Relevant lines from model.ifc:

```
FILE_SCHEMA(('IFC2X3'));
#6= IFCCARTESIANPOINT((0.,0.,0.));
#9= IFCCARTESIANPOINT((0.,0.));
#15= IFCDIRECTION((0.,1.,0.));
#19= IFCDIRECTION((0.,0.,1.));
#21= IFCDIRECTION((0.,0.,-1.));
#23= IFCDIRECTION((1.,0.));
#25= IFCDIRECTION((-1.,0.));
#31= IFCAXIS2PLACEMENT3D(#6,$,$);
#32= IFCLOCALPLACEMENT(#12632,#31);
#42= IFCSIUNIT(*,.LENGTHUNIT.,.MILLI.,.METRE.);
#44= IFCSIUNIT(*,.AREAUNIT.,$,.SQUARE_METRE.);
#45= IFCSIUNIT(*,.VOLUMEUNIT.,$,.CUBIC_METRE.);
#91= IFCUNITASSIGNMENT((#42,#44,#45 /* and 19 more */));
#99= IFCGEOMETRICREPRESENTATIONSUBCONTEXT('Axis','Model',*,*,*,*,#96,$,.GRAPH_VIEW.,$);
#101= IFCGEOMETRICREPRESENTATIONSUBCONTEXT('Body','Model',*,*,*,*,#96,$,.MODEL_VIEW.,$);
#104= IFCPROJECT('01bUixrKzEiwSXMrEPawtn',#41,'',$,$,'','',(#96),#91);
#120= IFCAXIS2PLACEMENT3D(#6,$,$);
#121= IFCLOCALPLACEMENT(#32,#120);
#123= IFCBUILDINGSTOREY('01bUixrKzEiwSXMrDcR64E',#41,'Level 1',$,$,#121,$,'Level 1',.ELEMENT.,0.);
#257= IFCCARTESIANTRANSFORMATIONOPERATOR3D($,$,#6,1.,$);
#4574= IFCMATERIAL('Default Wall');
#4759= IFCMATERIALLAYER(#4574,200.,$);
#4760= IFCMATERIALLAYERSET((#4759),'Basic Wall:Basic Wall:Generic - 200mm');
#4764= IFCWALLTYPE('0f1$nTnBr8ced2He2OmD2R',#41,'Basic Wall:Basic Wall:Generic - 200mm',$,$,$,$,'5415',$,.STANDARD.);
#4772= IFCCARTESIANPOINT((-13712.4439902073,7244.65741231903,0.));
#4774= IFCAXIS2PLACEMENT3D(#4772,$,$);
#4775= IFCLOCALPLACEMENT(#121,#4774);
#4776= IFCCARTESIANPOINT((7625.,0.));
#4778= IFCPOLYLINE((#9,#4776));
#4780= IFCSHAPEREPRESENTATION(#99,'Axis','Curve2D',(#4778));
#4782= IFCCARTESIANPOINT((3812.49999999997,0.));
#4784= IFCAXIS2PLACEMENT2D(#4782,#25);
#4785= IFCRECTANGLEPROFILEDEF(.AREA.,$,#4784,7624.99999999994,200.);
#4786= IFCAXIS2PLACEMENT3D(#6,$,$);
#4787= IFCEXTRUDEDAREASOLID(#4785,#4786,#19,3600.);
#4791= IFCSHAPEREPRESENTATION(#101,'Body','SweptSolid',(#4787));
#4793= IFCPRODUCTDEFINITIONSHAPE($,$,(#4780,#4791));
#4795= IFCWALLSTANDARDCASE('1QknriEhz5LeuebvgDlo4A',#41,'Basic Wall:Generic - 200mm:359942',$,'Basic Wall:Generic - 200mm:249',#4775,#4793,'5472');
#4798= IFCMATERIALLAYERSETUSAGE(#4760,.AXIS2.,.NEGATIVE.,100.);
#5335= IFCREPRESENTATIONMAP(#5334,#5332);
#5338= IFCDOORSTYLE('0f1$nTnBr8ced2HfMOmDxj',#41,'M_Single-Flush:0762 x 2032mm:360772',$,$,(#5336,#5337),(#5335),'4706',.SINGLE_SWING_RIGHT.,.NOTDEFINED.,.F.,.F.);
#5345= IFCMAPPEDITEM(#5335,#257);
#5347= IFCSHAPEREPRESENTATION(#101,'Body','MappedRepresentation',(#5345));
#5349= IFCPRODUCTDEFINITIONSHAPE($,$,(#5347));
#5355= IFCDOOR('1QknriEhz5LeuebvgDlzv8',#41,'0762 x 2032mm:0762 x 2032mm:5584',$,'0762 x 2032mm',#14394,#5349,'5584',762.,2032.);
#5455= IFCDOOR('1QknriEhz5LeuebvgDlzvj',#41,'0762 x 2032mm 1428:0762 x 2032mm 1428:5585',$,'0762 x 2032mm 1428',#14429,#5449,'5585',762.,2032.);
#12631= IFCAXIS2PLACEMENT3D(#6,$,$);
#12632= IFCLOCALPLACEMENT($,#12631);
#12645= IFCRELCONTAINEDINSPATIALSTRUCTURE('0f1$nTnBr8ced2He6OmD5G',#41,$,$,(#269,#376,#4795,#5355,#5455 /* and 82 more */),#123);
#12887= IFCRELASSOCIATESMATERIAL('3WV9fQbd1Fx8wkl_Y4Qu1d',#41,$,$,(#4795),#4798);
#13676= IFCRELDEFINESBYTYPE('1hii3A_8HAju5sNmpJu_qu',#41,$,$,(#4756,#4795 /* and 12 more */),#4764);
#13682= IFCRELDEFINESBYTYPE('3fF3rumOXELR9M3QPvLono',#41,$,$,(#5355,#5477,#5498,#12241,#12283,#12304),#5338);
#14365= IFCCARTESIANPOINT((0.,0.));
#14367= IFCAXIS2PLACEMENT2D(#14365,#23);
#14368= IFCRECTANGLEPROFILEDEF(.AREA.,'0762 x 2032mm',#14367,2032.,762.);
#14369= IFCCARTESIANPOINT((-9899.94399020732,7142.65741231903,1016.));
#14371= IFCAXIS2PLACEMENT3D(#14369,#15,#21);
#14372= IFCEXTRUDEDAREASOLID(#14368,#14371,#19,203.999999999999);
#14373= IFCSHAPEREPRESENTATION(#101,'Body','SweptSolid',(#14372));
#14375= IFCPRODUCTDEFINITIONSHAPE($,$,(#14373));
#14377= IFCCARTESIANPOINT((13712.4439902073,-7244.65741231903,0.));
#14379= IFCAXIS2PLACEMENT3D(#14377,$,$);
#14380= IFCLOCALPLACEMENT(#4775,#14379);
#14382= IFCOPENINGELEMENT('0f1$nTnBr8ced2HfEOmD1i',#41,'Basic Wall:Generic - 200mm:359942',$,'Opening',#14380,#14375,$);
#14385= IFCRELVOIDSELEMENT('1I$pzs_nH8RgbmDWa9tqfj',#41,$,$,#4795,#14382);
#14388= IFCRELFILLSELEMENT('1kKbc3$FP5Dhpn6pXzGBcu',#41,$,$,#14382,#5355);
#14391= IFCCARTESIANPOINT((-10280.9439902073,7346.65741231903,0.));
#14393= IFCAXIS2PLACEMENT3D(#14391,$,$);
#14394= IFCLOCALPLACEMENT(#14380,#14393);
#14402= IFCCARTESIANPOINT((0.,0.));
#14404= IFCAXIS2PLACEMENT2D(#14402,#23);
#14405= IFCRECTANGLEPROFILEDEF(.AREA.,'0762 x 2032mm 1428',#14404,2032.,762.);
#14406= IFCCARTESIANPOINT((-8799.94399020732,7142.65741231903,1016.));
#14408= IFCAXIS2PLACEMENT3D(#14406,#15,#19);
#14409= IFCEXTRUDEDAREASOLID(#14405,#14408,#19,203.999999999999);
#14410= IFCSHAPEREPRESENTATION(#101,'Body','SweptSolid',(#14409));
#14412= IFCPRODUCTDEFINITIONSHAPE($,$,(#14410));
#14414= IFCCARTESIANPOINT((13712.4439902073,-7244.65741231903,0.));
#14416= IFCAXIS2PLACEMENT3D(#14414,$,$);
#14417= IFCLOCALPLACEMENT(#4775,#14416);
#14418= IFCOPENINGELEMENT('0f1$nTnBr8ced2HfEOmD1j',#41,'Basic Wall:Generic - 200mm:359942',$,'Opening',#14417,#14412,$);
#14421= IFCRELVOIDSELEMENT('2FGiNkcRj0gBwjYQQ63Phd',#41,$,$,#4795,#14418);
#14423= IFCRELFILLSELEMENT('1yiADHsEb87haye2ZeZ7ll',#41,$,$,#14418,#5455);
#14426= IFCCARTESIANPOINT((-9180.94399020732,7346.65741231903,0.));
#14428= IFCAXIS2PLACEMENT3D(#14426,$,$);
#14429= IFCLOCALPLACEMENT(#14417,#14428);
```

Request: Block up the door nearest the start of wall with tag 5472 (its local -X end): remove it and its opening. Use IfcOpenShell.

```python
import ifcopenshell
import ifcopenshell.api.feature
import ifcopenshell.api.root
import ifcopenshell.geom
import ifcopenshell.util.shape

model = ifcopenshell.open("model.ifc")
settings = ifcopenshell.geom.settings()


def volume(element):
    """Net volume in cubic metres, openings subtracted."""
    shape = ifcopenshell.geom.create_shape(settings, element)
    return ifcopenshell.util.shape.get_volume(shape.geometry)


door = model.by_id(5355)
opening = door.FillsVoids[0].RelatingOpeningElement
wall = opening.VoidsElements[0].RelatingBuildingElement
before = volume(wall)

ifcopenshell.api.root.remove_product(model, product=door)
ifcopenshell.api.feature.remove_feature(model, feature=opening)

after = volume(wall)

print(f"wall volume {before:.3f} -> {after:.3f} m3")

model.write("model_updated.ifc")
```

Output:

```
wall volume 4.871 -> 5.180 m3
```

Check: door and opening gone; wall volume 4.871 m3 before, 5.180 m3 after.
